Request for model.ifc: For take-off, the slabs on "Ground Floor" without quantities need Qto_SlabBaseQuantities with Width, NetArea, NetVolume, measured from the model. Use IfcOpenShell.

First a look at what the model holds.

```python
import ifcopenshell
import ifcopenshell.util.element
import ifcopenshell.util.unit

model = ifcopenshell.open("model.ifc")
print(model.schema)
for unit_type in ("LENGTHUNIT", "AREAUNIT", "VOLUMEUNIT"):
    print(unit_type, ifcopenshell.util.unit.calculate_unit_scale(model, unit_type))
storey = next(s for s in model.by_type("IfcBuildingStorey") if s.Name == "Ground Floor")
slabs = [e for e in ifcopenshell.util.element.get_decomposition(storey) if e.is_a("IfcSlab")]
for e in sorted(slabs, key=lambda e: e.id()):
    print(e.id(), e.is_a(), e.Name, list(ifcopenshell.util.element.get_psets(e, qtos_only=True)), sep=" | ")
```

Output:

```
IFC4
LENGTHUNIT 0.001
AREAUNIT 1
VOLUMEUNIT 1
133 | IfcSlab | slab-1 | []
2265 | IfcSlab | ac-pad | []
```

```python
import ifcopenshell
import ifcopenshell.api.pset
import ifcopenshell.geom
import ifcopenshell.util.element
import ifcopenshell.util.shape
import ifcopenshell.util.unit

model = ifcopenshell.open("model.ifc")
unit_scale = ifcopenshell.util.unit.calculate_unit_scale(model)
area_scale = ifcopenshell.util.unit.calculate_unit_scale(model, "AREAUNIT")
volume_scale = ifcopenshell.util.unit.calculate_unit_scale(model, "VOLUMEUNIT")
settings = ifcopenshell.geom.settings()

storey = next(s for s in model.by_type("IfcBuildingStorey") if s.Name == "Ground Floor")
slabs = [e for e in ifcopenshell.util.element.get_decomposition(storey) if e.is_a("IfcSlab")]

for e in sorted(slabs, key=lambda e: e.id()):
    if ifcopenshell.util.element.get_psets(e, qtos_only=True, should_inherit=False):
        continue
    # Geometry comes back in metres, in the element's own axes.
    shape = ifcopenshell.geom.create_shape(settings, e)
    values = {
        "Width": ifcopenshell.util.shape.get_z(shape.geometry) / unit_scale,
        "NetArea": ifcopenshell.util.shape.get_footprint_area(shape.geometry) / area_scale,
        "NetVolume": ifcopenshell.util.shape.get_volume(shape.geometry) / volume_scale,
    }
    qto = ifcopenshell.api.pset.add_qto(model, product=e, name="Qto_SlabBaseQuantities")
    ifcopenshell.api.pset.edit_qto(model, qto=qto, properties=values)
    print(e.id(), {k: round(v, 3) for k, v in values.items()})

model.write("model_rev.ifc")
```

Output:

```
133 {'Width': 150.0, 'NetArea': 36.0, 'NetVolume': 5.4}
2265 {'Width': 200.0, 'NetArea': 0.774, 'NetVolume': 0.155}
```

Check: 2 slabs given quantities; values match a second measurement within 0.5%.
